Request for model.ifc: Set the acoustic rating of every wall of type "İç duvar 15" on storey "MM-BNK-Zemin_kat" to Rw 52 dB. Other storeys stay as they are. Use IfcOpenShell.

First a look at what the model holds.

```python
import ifcopenshell
import ifcopenshell.util.element

model = ifcopenshell.open("model.ifc")
print(model.schema)
storey = next(s for s in model.by_type("IfcBuildingStorey") if s.Name == "MM-BNK-Zemin_kat")
walls = [e for e in ifcopenshell.util.element.get_decomposition(storey) if e.is_a("IfcWall")]
seen = {}
for e in walls:
    element_type = ifcopenshell.util.element.get_type(e)
    key = (element_type.Name if element_type != e and element_type else None, ifcopenshell.util.element.get_pset(e, "Pset_WallCommon", "AcousticRating"))
    seen[key] = seen.get(key, 0) + 1
for (name, value), count in sorted(seen.items(), key=str):
    print(count, "x", name, "|", value)
```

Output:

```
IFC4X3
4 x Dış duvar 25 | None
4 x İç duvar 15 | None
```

```python
import ifcopenshell
import ifcopenshell.api.pset
import ifcopenshell.util.element

model = ifcopenshell.open("model.ifc")

storey = next(s for s in model.by_type("IfcBuildingStorey") if s.Name == "MM-BNK-Zemin_kat")
walls = [e for e in ifcopenshell.util.element.get_decomposition(storey) if e.is_a("IfcWall")]

count = 0
for e in walls:
    element_type = ifcopenshell.util.element.get_type(e)
    if element_type in (None, e) or element_type.Name != "İç duvar 15":
        continue
    # add_pset returns the element's existing set when there is one.
    pset = ifcopenshell.api.pset.add_pset(model, product=e, name="Pset_WallCommon")
    ifcopenshell.api.pset.edit_pset(model, pset=pset, properties={"AcousticRating": "Rw 52 dB"})
    count += 1

print(count, "walls updated")

model.write("model_edited.ifc")
```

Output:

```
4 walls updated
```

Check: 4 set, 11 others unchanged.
